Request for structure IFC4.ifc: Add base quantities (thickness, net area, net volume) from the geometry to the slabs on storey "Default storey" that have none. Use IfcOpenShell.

First a look at what the model holds.

```python
import ifcopenshell
import ifcopenshell.util.element
import ifcopenshell.util.unit

model = ifcopenshell.open("structure IFC4.ifc")
print(model.schema)
for unit_type in ("LENGTHUNIT", "AREAUNIT", "VOLUMEUNIT"):
    print(unit_type, ifcopenshell.util.unit.calculate_unit_scale(model, unit_type))
storey = next(s for s in model.by_type("IfcBuildingStorey") if s.Name == "Default storey")
slabs = [e for e in ifcopenshell.util.element.get_decomposition(storey) if e.is_a("IfcSlab")]
for e in sorted(slabs, key=lambda e: e.id()):
    print(e.id(), e.is_a(), e.Name, list(ifcopenshell.util.element.get_psets(e, qtos_only=True)), sep=" | ")
```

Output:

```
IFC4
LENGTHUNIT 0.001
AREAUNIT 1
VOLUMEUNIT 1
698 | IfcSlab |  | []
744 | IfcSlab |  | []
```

```python
import ifcopenshell
import ifcopenshell.api.pset
import ifcopenshell.geom
import ifcopenshell.util.element
import ifcopenshell.util.shape
import ifcopenshell.util.unit

model = ifcopenshell.open("structure IFC4.ifc")
unit_scale = ifcopenshell.util.unit.calculate_unit_scale(model)
area_scale = ifcopenshell.util.unit.calculate_unit_scale(model, "AREAUNIT")
volume_scale = ifcopenshell.util.unit.calculate_unit_scale(model, "VOLUMEUNIT")
settings = ifcopenshell.geom.settings()

storey = next(s for s in model.by_type("IfcBuildingStorey") if s.Name == "Default storey")
slabs = [e for e in ifcopenshell.util.element.get_decomposition(storey) if e.is_a("IfcSlab")]

for e in sorted(slabs, key=lambda e: e.id()):
    if ifcopenshell.util.element.get_psets(e, qtos_only=True, should_inherit=False):
        continue
    # Geometry comes back in metres, in the element's own axes.
    shape = ifcopenshell.geom.create_shape(settings, e)
    values = {
        "Width": ifcopenshell.util.shape.get_z(shape.geometry) / unit_scale,
        "NetArea": ifcopenshell.util.shape.get_footprint_area(shape.geometry) / area_scale,
        "NetVolume": ifcopenshell.util.shape.get_volume(shape.geometry) / volume_scale,
    }
    qto = ifcopenshell.api.pset.add_qto(model, product=e, name="Qto_SlabBaseQuantities")
    ifcopenshell.api.pset.edit_qto(model, qto=qto, properties=values)
    print(e.id(), {k: round(v, 3) for k, v in values.items()})

model.write("structure IFC4_rev.ifc")
```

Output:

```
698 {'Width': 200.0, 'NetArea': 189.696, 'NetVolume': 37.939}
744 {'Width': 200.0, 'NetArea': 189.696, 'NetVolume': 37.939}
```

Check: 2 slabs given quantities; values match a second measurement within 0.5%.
